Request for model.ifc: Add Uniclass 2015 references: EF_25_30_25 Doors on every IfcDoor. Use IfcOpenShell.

First a look at what the model holds.

```python
import ifcopenshell

model = ifcopenshell.open("model.ifc")
print(model.schema)
print("classifications:", [c.Name for c in model.by_type("IfcClassification")])
for ifc_class in ("IfcDoor", "IfcRoof", "IfcStair", "IfcWall", "IfcWindow"):
    print(ifc_class, len(model.by_type(ifc_class)))
```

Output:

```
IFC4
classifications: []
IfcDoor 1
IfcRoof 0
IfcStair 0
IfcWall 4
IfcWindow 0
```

```python
import ifcopenshell
import ifcopenshell.api.classification

model = ifcopenshell.open("model.ifc")

system = ifcopenshell.api.classification.add_classification(model, classification="Uniclass 2015")

codes = {
    "IfcDoor": ("EF_25_30_25", "Doors"),
}
for ifc_class, (code, name) in codes.items():
    products = model.by_type(ifc_class)
    ifcopenshell.api.classification.add_reference(
        model, products=products, classification=system, identification=code, name=name
    )
    print(code, len(products))

model.write("model_updated.ifc")
```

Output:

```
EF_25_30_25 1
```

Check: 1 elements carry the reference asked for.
